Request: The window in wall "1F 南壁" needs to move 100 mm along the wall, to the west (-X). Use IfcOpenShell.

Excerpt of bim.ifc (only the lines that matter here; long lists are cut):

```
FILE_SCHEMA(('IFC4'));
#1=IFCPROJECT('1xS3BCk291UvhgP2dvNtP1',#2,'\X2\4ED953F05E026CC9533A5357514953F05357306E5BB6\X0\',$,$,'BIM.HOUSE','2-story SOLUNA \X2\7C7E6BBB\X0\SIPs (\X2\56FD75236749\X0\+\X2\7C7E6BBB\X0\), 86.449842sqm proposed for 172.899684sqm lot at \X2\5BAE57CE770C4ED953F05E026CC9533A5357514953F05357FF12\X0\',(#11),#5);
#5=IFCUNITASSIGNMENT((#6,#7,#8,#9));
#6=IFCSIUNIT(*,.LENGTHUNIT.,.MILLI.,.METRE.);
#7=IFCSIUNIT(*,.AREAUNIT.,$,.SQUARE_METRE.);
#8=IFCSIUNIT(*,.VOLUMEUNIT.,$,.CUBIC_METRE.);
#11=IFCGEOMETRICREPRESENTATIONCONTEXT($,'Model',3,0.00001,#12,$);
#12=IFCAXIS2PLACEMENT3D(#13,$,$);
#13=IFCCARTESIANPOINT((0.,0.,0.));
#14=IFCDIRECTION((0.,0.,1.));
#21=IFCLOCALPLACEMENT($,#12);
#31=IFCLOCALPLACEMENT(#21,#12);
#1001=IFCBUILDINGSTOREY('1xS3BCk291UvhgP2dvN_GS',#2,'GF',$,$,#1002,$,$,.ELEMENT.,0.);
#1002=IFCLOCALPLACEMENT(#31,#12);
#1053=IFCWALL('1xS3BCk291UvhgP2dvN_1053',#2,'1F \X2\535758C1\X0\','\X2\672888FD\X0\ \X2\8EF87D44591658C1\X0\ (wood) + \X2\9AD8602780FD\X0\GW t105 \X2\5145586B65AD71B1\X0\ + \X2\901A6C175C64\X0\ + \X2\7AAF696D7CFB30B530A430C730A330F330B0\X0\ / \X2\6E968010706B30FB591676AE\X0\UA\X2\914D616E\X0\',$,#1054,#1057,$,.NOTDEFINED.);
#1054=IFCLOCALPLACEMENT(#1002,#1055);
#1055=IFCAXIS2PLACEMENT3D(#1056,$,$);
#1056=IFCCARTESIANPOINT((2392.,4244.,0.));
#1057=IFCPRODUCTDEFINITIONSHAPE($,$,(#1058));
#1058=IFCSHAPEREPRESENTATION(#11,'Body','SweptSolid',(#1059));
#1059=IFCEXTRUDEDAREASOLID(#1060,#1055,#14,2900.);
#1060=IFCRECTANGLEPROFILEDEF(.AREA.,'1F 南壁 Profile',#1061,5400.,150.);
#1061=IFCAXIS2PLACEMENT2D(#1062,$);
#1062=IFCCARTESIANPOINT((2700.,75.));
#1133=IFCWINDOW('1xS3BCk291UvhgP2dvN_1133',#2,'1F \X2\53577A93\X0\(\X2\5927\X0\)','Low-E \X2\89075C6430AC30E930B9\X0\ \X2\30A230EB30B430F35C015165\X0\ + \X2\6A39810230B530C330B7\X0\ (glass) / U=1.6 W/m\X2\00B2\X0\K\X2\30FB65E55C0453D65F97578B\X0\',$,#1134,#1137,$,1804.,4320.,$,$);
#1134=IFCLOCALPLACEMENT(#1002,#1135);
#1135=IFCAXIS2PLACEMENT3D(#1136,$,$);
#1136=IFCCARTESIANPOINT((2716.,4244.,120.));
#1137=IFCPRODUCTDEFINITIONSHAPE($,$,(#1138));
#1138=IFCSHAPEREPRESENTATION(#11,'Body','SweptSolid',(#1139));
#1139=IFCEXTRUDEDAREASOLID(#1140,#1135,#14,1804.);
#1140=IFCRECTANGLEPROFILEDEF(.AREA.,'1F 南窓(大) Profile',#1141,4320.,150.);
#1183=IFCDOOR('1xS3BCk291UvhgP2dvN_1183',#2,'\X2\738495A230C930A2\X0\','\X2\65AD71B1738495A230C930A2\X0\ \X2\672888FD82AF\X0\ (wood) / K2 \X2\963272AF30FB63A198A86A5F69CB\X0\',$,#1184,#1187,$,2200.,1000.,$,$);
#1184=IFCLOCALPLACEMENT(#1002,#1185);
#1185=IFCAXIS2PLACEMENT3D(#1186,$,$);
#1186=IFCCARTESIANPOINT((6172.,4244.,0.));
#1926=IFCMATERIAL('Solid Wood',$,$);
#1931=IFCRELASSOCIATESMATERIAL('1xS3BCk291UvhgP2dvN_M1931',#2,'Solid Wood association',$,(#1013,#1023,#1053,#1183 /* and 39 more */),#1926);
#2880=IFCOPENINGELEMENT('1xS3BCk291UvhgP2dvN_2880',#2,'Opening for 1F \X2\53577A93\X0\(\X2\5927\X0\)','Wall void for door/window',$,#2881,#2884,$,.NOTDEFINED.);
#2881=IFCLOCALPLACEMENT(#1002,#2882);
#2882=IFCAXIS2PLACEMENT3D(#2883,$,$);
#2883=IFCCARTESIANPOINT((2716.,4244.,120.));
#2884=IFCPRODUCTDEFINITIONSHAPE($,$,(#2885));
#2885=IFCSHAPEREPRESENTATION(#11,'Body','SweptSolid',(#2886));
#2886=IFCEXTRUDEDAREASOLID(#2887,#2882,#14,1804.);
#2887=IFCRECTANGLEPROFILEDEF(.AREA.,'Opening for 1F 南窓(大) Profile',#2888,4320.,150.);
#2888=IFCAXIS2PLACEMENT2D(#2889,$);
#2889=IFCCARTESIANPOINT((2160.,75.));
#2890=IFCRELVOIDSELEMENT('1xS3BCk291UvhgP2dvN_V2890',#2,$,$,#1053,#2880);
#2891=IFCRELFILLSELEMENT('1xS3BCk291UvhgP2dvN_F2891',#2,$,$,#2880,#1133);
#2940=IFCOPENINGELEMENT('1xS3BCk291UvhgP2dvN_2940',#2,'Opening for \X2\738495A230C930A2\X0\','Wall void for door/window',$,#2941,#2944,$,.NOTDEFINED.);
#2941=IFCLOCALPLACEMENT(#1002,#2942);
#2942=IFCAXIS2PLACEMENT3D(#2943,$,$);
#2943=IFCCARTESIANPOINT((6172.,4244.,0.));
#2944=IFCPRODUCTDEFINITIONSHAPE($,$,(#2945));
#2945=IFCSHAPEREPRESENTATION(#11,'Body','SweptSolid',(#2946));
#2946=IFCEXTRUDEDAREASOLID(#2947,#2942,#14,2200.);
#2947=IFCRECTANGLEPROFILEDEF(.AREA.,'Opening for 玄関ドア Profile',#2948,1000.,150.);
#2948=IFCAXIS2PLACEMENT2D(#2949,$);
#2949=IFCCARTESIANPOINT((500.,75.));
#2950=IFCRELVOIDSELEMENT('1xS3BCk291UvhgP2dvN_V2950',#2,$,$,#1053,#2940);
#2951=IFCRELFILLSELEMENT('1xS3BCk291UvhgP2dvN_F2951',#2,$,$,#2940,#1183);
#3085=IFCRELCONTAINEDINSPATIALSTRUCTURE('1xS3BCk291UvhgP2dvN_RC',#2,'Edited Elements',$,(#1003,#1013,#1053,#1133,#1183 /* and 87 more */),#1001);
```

```python
import ifcopenshell
import ifcopenshell.api.geometry
import ifcopenshell.util.placement
import ifcopenshell.util.unit

model = ifcopenshell.open("bim.ifc")
unit_scale = ifcopenshell.util.unit.calculate_unit_scale(model)

window = model.by_guid("1xS3BCk291UvhgP2dvN_1133")
opening = window.FillsVoids[0].RelatingOpeningElement
wall = opening.VoidsElements[0].RelatingBuildingElement

wall_matrix = ifcopenshell.util.placement.get_local_placement(wall.ObjectPlacement)
shift = wall_matrix[:3, 0] * -0.1 / unit_scale
before = ifcopenshell.util.placement.get_local_placement(window.ObjectPlacement)[:3, 3].copy()

# The window is not placed relative to its opening, so move both.
for product in (opening, window):
    matrix = ifcopenshell.util.placement.get_local_placement(product.ObjectPlacement)
    matrix[:3, 3] += shift
    ifcopenshell.api.geometry.edit_object_placement(model, product=product, matrix=matrix, is_si=False)

after = ifcopenshell.util.placement.get_local_placement(window.ObjectPlacement)[:3, 3]
print("window moved by", (after - before).round(3) + 0.0)

model.write("bim_updated.ifc")
```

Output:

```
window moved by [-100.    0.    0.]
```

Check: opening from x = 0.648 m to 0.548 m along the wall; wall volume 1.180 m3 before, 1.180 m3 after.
